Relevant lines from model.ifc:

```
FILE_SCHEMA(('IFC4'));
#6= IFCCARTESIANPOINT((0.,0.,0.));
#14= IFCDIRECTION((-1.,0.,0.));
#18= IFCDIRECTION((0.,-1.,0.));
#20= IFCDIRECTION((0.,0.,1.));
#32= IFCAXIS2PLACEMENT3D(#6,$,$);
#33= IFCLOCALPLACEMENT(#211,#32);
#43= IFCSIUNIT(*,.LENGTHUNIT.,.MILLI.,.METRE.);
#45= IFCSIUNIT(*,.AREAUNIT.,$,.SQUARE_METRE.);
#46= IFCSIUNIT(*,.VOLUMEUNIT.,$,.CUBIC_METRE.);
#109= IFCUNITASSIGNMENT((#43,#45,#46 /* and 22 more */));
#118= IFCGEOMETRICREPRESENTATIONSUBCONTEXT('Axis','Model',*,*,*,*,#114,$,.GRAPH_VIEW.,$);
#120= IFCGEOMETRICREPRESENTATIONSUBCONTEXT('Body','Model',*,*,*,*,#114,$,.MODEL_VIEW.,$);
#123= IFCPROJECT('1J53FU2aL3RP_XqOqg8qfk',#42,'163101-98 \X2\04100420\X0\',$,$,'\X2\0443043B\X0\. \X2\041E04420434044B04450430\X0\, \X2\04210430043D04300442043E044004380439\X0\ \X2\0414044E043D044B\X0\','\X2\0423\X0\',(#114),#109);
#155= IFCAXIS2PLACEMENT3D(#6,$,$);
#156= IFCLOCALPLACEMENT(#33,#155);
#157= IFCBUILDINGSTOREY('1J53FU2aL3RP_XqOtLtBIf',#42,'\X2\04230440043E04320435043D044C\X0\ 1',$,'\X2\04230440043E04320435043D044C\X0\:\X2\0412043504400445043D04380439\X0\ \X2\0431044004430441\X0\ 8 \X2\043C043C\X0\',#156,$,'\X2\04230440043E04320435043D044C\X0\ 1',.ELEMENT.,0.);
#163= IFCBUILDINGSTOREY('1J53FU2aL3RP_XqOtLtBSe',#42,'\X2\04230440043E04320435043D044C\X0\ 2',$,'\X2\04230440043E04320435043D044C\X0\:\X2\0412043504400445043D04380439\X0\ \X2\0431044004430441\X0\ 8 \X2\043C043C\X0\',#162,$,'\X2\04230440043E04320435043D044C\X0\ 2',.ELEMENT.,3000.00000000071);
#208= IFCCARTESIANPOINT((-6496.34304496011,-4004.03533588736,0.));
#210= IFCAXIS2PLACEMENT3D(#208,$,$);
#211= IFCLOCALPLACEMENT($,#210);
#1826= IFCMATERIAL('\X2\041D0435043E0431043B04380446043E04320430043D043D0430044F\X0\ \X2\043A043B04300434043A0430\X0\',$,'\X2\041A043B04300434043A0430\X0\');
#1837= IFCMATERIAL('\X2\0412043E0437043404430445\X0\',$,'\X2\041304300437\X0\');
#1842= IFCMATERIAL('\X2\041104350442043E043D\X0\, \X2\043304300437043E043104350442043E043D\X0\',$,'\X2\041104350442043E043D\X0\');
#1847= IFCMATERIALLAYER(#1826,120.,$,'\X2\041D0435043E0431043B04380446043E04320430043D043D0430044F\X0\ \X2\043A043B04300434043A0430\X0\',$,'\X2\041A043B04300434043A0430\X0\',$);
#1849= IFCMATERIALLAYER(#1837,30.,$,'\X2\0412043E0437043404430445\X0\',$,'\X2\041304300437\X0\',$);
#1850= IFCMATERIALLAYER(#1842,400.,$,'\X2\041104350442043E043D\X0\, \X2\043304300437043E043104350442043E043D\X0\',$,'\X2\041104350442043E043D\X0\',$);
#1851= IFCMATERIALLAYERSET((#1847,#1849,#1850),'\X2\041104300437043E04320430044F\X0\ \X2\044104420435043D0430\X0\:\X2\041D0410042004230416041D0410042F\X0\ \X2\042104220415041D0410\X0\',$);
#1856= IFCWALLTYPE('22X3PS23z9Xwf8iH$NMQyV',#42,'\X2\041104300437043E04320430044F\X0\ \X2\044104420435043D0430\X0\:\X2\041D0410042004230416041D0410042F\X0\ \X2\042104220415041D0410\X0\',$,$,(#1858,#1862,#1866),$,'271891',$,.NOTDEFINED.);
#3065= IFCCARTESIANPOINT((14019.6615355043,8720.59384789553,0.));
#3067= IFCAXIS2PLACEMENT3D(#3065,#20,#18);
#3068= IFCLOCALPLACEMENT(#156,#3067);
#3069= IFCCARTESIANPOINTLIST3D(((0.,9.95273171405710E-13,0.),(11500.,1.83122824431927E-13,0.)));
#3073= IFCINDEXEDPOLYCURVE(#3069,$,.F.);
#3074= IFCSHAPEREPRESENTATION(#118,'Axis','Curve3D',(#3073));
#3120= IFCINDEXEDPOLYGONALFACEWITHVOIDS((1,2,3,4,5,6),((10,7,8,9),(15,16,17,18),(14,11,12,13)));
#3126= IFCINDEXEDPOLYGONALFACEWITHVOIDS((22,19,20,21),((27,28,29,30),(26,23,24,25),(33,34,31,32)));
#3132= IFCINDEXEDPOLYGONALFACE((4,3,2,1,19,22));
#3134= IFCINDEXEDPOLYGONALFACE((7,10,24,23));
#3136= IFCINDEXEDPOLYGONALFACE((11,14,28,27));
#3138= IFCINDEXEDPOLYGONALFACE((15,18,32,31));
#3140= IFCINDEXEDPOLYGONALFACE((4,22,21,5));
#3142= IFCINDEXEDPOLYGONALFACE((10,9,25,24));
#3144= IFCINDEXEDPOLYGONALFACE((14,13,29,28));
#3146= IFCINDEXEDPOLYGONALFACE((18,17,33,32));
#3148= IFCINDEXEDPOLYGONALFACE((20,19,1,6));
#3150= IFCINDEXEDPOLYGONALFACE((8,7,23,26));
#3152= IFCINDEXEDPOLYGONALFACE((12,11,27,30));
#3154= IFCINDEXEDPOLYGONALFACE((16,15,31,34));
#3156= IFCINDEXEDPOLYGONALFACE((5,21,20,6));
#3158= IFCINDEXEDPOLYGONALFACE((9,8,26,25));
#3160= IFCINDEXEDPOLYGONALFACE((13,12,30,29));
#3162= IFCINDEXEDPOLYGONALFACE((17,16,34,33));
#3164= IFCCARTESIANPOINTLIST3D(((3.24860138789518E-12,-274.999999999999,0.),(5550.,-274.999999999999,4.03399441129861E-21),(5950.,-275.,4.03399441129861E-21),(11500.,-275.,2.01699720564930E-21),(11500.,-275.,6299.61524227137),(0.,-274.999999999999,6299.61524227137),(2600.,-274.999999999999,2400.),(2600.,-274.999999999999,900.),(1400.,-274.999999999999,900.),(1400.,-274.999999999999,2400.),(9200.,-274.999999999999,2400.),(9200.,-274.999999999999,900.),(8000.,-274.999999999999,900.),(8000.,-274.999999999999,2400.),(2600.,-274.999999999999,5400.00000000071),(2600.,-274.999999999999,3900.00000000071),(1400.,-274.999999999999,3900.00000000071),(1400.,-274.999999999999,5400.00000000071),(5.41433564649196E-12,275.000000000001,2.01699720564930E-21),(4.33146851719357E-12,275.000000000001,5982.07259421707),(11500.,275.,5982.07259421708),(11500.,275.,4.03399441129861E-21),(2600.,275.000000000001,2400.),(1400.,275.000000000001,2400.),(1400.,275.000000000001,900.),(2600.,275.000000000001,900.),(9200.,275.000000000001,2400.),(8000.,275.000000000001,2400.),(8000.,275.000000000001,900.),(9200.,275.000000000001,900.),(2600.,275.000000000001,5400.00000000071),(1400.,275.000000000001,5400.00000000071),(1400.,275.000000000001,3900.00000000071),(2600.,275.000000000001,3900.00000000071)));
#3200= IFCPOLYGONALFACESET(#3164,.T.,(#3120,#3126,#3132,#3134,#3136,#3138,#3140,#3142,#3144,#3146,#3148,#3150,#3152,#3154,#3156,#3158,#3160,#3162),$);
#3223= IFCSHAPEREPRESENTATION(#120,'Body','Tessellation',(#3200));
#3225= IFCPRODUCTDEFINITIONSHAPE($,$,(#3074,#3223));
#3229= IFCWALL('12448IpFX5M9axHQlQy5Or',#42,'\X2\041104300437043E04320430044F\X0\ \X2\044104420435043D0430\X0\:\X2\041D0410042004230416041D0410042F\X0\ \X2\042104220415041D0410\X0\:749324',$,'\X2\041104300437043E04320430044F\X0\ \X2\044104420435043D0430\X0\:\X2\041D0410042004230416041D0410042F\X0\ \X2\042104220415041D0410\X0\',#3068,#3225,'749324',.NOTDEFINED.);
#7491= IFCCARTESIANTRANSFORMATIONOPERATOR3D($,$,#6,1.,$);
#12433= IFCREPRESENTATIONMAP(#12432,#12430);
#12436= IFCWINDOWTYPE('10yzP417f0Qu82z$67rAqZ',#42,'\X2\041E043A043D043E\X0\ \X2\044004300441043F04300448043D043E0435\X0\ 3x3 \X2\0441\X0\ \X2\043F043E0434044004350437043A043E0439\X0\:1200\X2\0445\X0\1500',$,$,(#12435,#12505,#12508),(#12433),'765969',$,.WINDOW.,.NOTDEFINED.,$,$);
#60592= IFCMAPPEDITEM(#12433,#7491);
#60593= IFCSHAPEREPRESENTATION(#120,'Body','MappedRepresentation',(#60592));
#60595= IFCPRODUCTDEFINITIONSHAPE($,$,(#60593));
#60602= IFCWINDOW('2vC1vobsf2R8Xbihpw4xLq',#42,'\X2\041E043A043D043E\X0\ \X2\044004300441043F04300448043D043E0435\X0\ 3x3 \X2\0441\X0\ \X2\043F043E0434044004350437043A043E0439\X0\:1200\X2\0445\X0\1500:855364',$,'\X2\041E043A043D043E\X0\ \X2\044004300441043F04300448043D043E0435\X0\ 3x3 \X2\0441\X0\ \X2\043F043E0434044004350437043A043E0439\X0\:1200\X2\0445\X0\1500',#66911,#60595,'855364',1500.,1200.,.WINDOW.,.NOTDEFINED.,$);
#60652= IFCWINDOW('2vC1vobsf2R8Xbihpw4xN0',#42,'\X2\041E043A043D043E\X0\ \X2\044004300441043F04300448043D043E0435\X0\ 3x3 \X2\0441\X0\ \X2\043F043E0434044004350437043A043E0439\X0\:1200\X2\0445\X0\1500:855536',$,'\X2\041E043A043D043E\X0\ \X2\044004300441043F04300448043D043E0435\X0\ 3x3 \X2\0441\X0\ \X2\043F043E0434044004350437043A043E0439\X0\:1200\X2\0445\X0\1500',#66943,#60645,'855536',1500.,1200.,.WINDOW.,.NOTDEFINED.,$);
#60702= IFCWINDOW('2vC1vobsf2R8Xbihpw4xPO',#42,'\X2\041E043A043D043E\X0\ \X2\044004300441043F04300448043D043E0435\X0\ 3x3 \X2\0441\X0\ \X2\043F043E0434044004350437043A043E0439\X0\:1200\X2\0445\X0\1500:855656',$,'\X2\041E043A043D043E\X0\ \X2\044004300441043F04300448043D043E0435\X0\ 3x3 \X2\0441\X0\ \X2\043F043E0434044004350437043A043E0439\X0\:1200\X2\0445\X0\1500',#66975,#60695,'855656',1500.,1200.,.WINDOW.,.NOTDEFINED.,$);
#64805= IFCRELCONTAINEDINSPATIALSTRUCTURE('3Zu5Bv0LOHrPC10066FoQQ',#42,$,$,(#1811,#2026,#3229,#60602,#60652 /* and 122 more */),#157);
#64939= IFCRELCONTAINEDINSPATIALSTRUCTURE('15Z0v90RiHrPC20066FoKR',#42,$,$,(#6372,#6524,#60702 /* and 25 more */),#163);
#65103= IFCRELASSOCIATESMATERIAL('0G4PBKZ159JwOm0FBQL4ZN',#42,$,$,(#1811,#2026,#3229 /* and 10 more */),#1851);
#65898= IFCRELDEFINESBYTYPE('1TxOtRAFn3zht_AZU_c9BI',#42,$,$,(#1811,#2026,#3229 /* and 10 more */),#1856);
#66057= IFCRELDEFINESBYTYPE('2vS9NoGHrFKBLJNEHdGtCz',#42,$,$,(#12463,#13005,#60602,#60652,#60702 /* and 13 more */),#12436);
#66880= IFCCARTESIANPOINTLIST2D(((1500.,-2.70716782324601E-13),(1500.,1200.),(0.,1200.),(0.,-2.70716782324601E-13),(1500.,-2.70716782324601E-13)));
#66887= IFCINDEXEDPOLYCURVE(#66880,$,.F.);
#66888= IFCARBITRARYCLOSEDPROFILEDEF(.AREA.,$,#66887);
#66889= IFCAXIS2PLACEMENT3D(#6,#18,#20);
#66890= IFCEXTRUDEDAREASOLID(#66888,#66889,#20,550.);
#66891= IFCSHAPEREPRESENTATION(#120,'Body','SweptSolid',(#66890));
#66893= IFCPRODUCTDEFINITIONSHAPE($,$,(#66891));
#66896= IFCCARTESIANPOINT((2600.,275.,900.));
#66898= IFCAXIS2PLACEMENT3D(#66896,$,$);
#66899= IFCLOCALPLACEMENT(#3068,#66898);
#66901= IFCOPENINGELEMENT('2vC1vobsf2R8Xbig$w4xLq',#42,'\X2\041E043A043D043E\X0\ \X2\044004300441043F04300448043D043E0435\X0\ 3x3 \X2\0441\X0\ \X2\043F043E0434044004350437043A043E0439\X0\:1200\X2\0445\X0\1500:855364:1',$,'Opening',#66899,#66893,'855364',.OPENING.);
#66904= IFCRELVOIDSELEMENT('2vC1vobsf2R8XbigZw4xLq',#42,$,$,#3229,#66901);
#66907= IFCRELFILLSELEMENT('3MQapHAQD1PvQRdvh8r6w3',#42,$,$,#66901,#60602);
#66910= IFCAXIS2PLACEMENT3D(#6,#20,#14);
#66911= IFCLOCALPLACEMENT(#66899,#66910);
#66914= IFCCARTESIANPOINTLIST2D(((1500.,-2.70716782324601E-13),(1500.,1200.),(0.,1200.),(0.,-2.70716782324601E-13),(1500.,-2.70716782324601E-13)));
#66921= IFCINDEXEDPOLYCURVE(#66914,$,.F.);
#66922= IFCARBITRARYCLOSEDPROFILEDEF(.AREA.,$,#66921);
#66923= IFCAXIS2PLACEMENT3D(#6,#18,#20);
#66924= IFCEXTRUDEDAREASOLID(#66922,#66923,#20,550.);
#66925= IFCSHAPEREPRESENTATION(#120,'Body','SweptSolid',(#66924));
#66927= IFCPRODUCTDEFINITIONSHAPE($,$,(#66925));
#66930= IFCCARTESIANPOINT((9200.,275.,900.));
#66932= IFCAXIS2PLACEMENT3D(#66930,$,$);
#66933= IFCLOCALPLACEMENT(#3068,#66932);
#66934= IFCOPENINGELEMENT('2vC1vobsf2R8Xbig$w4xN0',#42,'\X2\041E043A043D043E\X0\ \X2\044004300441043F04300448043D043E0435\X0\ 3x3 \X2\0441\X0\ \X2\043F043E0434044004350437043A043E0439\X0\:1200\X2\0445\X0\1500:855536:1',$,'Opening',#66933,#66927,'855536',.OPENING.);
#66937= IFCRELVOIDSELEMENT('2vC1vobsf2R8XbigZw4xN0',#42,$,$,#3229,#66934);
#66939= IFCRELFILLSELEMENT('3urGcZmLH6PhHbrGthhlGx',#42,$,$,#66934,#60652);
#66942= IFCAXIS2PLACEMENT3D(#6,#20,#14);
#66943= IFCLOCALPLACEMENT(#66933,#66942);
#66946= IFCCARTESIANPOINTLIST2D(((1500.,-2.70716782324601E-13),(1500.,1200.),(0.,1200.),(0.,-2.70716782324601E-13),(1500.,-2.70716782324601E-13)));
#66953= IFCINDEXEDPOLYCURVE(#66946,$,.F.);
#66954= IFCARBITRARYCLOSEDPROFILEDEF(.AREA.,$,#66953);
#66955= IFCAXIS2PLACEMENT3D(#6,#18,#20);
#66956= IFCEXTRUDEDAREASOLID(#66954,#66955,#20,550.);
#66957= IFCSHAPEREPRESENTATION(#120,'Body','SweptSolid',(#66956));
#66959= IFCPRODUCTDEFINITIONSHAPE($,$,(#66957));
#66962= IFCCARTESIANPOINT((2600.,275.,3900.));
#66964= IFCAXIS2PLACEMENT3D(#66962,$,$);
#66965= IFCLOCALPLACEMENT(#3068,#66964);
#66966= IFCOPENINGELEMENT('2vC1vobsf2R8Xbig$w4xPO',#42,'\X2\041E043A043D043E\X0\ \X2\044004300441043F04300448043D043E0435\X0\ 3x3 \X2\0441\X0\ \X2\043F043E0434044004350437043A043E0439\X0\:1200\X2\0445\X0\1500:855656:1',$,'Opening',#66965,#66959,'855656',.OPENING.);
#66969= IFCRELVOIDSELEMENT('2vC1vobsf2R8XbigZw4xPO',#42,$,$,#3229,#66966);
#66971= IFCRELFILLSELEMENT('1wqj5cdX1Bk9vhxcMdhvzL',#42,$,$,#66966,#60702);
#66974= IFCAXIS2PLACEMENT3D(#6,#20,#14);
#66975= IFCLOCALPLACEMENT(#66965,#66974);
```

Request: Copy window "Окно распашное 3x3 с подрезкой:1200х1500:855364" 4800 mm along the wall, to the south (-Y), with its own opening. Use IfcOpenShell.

```python
import ifcopenshell
import ifcopenshell.api.feature
import ifcopenshell.api.geometry
import ifcopenshell.api.root
import ifcopenshell.geom
import ifcopenshell.util.element
import ifcopenshell.util.placement
import ifcopenshell.util.shape
import ifcopenshell.util.unit

model = ifcopenshell.open("model.ifc")
unit_scale = ifcopenshell.util.unit.calculate_unit_scale(model)
settings = ifcopenshell.geom.settings()


def volume(element):
    """Net volume in cubic metres, openings subtracted."""
    shape = ifcopenshell.geom.create_shape(settings, element)
    return ifcopenshell.util.shape.get_volume(shape.geometry)


def reuse_history(source, copy):
    """copy_class also copies each property set's owner history, people and application; keep the originals."""
    for rel in copy.IsDefinedBy:
        if rel.is_a("IfcRelDefinesByProperties") and (history := rel.RelatingPropertyDefinition.OwnerHistory):
            rel.RelatingPropertyDefinition.OwnerHistory = source.OwnerHistory
            ifcopenshell.util.element.remove_deep2(model, history)


window = model.by_guid("2vC1vobsf2R8Xbihpw4xLq")
opening = window.FillsVoids[0].RelatingOpeningElement
wall = opening.VoidsElements[0].RelatingBuildingElement
before = volume(wall)
shift = ifcopenshell.util.placement.get_local_placement(wall.ObjectPlacement)[:3, 0] * 4.8 / unit_scale

# copy_class copies the void relationship, type, container and properties, but no geometry.
new_opening = ifcopenshell.api.root.copy_class(model, product=opening)
new_opening.Representation = ifcopenshell.util.element.copy_deep(
    model, opening.Representation, exclude=["IfcGeometricRepresentationContext", "IfcRepresentationMap"]
)
new_opening.Name = "Окно распашное 3x3 с подрезкой:1200х1500"
new_opening.Tag = None
new_window = ifcopenshell.api.root.copy_class(model, product=window)
new_window.Representation = ifcopenshell.util.element.copy_deep(
    model, window.Representation, exclude=["IfcGeometricRepresentationContext", "IfcRepresentationMap"]
)
new_window.Name = "Окно распашное 3x3 с подрезкой:1200х1500"
new_window.Tag = None
reuse_history(window, new_window)
ifcopenshell.api.feature.add_filling(model, opening=new_opening, element=new_window)

for old, new in ((opening, new_opening), (window, new_window)):
    matrix = ifcopenshell.util.placement.get_local_placement(old.ObjectPlacement)
    matrix[:3, 3] += shift
    ifcopenshell.api.geometry.edit_object_placement(model, product=new, matrix=matrix, is_si=False)

after = volume(wall)

print(f"wall volume {before:.3f} -> {after:.3f} m3")

model.write("model-out.ifc")
```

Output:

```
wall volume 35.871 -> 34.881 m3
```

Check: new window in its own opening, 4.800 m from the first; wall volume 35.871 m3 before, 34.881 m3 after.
